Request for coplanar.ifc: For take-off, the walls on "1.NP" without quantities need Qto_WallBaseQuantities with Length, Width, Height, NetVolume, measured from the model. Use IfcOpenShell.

First a look at what the model holds.

```python
import ifcopenshell
import ifcopenshell.util.element
import ifcopenshell.util.unit

model = ifcopenshell.open("coplanar.ifc")
print(model.schema)
for unit_type in ("LENGTHUNIT", "AREAUNIT", "VOLUMEUNIT"):
    print(unit_type, ifcopenshell.util.unit.calculate_unit_scale(model, unit_type))
storey = next(s for s in model.by_type("IfcBuildingStorey") if s.Name == "1.NP")
walls = [e for e in ifcopenshell.util.element.get_decomposition(storey) if e.is_a("IfcWall")]
for e in sorted(walls, key=lambda e: e.id()):
    print(e.id(), e.is_a(), e.Name, list(ifcopenshell.util.element.get_psets(e, qtos_only=True)), sep=" | ")
```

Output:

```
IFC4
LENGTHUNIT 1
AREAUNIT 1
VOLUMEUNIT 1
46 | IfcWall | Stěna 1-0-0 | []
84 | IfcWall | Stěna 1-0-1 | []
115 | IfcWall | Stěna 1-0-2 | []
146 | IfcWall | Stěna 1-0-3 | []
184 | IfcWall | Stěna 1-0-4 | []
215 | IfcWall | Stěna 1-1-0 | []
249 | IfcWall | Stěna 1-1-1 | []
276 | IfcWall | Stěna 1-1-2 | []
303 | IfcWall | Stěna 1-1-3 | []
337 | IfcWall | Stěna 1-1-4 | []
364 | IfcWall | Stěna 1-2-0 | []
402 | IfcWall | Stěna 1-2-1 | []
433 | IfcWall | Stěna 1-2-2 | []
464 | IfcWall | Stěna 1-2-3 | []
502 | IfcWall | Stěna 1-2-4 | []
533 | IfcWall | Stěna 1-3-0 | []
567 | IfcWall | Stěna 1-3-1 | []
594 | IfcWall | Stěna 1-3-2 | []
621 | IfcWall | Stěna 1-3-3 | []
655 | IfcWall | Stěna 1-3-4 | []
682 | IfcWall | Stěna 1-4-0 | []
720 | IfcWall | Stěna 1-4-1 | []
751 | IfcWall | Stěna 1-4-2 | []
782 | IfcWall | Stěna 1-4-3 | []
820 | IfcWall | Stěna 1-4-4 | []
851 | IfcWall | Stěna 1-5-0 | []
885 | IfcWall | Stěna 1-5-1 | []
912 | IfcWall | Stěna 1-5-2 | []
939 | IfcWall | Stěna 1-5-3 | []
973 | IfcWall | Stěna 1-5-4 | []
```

```python
import ifcopenshell
import ifcopenshell.api.pset
import ifcopenshell.geom
import ifcopenshell.util.element
import ifcopenshell.util.shape
import ifcopenshell.util.unit

model = ifcopenshell.open("coplanar.ifc")
unit_scale = ifcopenshell.util.unit.calculate_unit_scale(model)
volume_scale = ifcopenshell.util.unit.calculate_unit_scale(model, "VOLUMEUNIT")
settings = ifcopenshell.geom.settings()

storey = next(s for s in model.by_type("IfcBuildingStorey") if s.Name == "1.NP")
walls = [e for e in ifcopenshell.util.element.get_decomposition(storey) if e.is_a("IfcWall")]

for e in sorted(walls, key=lambda e: e.id()):
    if ifcopenshell.util.element.get_psets(e, qtos_only=True, should_inherit=False):
        continue
    # Geometry comes back in metres, in the element's own axes.
    shape = ifcopenshell.geom.create_shape(settings, e)
    values = {
        "Length": ifcopenshell.util.shape.get_x(shape.geometry) / unit_scale,
        "Width": ifcopenshell.util.shape.get_y(shape.geometry) / unit_scale,
        "Height": ifcopenshell.util.shape.get_z(shape.geometry) / unit_scale,
        "NetVolume": ifcopenshell.util.shape.get_volume(shape.geometry) / volume_scale,
    }
    qto = ifcopenshell.api.pset.add_qto(model, product=e, name="Qto_WallBaseQuantities")
    ifcopenshell.api.pset.edit_qto(model, qto=qto, properties=values)
    print(e.id(), {k: round(v, 3) for k, v in values.items()})

model.write("coplanar_updated.ifc")
```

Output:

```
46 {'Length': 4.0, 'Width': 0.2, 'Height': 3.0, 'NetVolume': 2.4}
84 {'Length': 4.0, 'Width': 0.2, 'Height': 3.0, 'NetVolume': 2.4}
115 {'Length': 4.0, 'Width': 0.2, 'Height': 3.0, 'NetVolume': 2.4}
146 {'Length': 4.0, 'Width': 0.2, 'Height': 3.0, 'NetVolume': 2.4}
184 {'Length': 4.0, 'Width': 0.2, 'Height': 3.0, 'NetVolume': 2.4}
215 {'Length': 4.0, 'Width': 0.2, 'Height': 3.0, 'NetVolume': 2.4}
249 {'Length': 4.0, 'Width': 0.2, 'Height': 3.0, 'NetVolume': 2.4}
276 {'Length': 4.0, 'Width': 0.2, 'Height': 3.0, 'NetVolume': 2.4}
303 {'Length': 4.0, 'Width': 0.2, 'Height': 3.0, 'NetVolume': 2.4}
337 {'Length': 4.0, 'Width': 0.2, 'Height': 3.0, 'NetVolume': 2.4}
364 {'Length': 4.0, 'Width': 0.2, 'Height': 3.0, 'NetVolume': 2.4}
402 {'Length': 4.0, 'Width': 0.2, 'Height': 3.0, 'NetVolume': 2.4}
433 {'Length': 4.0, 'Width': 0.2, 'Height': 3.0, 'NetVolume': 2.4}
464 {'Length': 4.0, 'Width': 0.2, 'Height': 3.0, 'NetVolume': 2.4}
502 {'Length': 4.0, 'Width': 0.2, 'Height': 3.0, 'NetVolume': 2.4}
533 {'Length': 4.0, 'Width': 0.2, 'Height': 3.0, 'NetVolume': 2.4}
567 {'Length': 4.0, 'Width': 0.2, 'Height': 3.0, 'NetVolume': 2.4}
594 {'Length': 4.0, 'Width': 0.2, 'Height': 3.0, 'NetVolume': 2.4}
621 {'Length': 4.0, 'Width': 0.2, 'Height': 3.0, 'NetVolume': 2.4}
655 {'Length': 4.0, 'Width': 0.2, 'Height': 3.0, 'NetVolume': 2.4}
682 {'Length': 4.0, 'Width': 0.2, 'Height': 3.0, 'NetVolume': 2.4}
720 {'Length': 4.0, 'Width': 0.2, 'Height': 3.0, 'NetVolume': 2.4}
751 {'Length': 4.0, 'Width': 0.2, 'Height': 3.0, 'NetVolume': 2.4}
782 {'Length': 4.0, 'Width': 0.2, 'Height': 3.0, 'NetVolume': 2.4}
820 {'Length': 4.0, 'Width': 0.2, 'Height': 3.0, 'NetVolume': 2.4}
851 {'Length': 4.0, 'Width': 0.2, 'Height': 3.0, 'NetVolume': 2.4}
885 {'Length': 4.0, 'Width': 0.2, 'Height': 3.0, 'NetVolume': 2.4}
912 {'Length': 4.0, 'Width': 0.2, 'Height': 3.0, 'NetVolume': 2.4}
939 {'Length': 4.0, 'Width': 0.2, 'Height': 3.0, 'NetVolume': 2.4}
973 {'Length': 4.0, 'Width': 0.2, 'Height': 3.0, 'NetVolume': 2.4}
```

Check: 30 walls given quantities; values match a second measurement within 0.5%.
